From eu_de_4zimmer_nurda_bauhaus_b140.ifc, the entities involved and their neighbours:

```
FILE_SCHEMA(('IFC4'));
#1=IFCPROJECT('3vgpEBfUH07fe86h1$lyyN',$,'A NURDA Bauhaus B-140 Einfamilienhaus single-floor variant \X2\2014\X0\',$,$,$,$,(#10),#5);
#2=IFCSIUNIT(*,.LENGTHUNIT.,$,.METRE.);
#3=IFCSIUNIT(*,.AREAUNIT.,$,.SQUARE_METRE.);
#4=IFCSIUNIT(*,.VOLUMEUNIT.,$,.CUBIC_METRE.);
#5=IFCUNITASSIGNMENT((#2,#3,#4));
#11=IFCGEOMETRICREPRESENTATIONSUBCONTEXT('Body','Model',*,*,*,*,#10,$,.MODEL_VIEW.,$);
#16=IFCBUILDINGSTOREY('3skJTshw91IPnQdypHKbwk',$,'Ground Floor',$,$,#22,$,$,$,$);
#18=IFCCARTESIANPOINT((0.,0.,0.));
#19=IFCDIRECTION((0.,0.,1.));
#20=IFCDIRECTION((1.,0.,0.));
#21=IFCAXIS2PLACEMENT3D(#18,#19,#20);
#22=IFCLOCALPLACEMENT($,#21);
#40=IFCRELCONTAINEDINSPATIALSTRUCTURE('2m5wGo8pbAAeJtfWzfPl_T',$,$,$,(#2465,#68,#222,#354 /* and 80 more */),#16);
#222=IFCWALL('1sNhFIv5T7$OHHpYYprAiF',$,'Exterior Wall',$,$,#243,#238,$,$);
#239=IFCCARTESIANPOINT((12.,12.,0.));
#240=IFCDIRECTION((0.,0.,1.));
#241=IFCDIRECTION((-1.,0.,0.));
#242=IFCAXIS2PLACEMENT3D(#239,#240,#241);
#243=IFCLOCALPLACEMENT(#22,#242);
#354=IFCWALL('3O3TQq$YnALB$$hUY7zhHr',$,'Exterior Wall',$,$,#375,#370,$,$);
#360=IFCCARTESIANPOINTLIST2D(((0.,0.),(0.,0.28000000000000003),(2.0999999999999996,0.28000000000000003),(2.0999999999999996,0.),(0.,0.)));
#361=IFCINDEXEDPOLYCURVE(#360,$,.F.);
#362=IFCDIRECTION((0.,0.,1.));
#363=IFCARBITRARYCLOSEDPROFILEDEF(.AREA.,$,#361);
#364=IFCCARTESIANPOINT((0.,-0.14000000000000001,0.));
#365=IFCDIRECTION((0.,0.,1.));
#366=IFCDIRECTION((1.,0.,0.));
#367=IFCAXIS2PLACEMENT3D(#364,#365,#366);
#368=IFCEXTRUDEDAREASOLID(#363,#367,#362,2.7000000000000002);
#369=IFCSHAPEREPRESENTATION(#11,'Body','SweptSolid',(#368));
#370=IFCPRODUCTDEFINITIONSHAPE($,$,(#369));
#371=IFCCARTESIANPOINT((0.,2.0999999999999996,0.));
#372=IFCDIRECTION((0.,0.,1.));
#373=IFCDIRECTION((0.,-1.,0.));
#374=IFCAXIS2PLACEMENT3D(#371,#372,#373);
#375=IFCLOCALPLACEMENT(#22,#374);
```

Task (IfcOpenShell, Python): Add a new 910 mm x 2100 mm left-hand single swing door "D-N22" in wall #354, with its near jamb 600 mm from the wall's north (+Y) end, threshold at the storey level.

```python
import numpy as np
import ifcopenshell
import ifcopenshell.api.feature
import ifcopenshell.api.geometry
import ifcopenshell.api.root
import ifcopenshell.api.spatial
import ifcopenshell.geom
import ifcopenshell.util.element
import ifcopenshell.util.placement
import ifcopenshell.util.representation
import ifcopenshell.util.shape
import ifcopenshell.util.unit

model = ifcopenshell.open("eu_de_4zimmer_nurda_bauhaus_b140.ifc")
unit_scale = ifcopenshell.util.unit.calculate_unit_scale(model)
settings = ifcopenshell.geom.settings()


def volume(element):
    """Net volume in cubic metres, openings subtracted."""
    shape = ifcopenshell.geom.create_shape(settings, element)
    return ifcopenshell.util.shape.get_volume(shape.geometry)


wall = model.by_id(354)
storey = ifcopenshell.util.element.get_container(wall, ifc_class="IfcBuildingStorey")
context = ifcopenshell.util.representation.get_context(model, "Model", "Body", "MODEL_VIEW")
before = volume(wall)

width, height, from_end, sill = 0.91, 2.1, 0.6, 0.0  # metres

# The wall runs along its own X axis, and the end named is its -X end.
wall_shape = ifcopenshell.geom.create_shape(settings, wall)
x, y, z = ifcopenshell.util.shape.get_vertices(wall_shape.geometry).T
start = x.min() + from_end
face, thickness = float(y.min()), float(y.max() - y.min())
wall_matrix = ifcopenshell.util.placement.get_local_placement(wall.ObjectPlacement)
level = ifcopenshell.util.placement.get_local_placement(storey.ObjectPlacement)[2, 3]


def in_wall(x, y):
    """Placement at x, y metres in the wall's axes, at sill height."""
    matrix = wall_matrix.copy()
    matrix[:, 3] = wall_matrix @ np.array([x / unit_scale, y / unit_scale, 0.0, 1.0])
    matrix[2, 3] = level + sill / unit_scale
    return matrix


# Opening: a box that overshoots both wall faces by 50 mm.
opening = ifcopenshell.api.root.create_entity(model, ifc_class="IfcOpeningElement", predefined_type="OPENING")
box = ifcopenshell.api.geometry.add_wall_representation(
    model, context=context, length=width, height=height, thickness=thickness + 0.1
)
ifcopenshell.api.geometry.assign_representation(model, product=opening, representation=box)
ifcopenshell.api.geometry.edit_object_placement(model, product=opening, matrix=in_wall(start, face - 0.05), is_si=False)
ifcopenshell.api.feature.add_feature(model, feature=opening, element=wall)

door = ifcopenshell.api.root.create_entity(model, ifc_class="IfcDoor", name="D-N22", predefined_type="DOOR")
door.OverallWidth, door.OverallHeight = width / unit_scale, height / unit_scale
door.OperationType = "SINGLE_SWING_LEFT"
body = ifcopenshell.api.geometry.add_door_representation(
    model,
    context=context,
    overall_width=door.OverallWidth,
    overall_height=door.OverallHeight,
    operation_type="SINGLE_SWING_LEFT",
    lining_properties={"LiningDepth": thickness / unit_scale, "ThresholdDepth": thickness / unit_scale},
)
ifcopenshell.api.geometry.assign_representation(model, product=door, representation=body)
ifcopenshell.api.spatial.assign_container(model, products=[door], relating_structure=storey)
ifcopenshell.api.feature.add_filling(model, opening=opening, element=door)

# The lining spans the wall, so the door starts at the wall face.
ifcopenshell.api.geometry.edit_object_placement(model, product=door, matrix=in_wall(start, face), is_si=False)

after = volume(wall)

print(f"wall volume {before:.3f} -> {after:.3f} m3")

model.write("eu_de_4zimmer_nurda_bauhaus_b140_updated.ifc")
```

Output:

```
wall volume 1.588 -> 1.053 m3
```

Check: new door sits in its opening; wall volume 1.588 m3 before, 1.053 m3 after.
